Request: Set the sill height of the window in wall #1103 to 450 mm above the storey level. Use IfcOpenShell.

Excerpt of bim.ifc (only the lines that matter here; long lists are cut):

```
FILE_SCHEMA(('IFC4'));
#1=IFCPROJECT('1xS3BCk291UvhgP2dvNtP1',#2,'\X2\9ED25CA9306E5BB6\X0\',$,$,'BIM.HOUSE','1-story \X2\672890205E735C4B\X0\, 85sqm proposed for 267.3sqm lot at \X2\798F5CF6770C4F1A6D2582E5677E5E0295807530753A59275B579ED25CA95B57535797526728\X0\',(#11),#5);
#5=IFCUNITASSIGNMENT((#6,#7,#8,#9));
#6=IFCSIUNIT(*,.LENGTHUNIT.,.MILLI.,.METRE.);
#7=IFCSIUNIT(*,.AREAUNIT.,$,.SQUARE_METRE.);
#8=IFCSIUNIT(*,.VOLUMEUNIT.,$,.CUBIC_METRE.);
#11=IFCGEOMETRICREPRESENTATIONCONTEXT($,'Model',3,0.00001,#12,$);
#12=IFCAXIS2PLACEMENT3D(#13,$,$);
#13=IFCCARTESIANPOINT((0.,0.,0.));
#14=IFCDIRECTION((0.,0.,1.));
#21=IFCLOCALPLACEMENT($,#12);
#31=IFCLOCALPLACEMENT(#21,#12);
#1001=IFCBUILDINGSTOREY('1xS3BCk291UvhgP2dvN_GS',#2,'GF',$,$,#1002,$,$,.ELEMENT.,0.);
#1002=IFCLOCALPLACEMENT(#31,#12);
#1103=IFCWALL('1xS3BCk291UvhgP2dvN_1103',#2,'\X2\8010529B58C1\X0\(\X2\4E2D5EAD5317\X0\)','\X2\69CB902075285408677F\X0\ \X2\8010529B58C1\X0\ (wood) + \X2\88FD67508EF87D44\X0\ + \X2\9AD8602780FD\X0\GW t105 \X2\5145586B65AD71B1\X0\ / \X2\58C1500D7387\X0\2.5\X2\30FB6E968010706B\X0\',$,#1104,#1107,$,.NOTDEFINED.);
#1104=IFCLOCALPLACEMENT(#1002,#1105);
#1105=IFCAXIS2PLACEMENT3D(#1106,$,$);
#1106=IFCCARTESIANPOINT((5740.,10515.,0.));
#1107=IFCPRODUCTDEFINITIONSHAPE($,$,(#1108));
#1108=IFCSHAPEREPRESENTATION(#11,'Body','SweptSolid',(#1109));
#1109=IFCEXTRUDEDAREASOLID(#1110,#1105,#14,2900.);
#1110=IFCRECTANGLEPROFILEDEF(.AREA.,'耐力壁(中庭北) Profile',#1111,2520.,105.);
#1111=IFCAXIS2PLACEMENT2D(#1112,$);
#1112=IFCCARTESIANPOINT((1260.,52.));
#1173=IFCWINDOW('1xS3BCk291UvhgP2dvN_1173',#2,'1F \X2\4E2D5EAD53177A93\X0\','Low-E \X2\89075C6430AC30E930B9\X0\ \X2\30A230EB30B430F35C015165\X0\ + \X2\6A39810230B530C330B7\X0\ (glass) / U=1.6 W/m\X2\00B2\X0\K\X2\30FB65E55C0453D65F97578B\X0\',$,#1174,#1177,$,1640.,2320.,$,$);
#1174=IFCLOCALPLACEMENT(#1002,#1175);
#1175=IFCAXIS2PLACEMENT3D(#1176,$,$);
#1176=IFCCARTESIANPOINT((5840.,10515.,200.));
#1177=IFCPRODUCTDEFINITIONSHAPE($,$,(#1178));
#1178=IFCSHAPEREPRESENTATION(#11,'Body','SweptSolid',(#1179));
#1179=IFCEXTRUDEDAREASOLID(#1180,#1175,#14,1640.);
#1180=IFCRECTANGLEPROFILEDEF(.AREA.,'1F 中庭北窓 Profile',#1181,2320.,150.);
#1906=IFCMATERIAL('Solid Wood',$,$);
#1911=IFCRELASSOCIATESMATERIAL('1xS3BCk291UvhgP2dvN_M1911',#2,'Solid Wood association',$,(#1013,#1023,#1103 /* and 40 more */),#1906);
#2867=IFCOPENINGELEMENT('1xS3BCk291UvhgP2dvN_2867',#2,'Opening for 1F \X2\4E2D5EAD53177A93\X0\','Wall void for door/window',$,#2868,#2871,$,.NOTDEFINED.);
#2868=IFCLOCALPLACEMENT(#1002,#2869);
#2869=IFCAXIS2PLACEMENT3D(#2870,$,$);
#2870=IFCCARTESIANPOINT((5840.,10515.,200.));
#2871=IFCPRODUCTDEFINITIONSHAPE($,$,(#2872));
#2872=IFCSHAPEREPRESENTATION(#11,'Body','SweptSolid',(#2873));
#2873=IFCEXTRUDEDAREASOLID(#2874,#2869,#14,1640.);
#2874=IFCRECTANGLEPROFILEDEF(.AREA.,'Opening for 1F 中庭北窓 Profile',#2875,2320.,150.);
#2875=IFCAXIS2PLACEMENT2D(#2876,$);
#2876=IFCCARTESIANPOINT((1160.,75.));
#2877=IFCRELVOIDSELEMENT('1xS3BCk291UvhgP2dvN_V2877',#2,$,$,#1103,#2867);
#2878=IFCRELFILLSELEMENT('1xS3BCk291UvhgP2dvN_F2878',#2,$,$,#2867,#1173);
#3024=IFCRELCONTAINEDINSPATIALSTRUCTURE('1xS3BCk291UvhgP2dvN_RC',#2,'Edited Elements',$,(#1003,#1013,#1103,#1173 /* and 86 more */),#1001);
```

```python
import numpy as np
import ifcopenshell
import ifcopenshell.api.geometry
import ifcopenshell.geom
import ifcopenshell.util.element
import ifcopenshell.util.placement
import ifcopenshell.util.shape
import ifcopenshell.util.unit

model = ifcopenshell.open("bim.ifc")
unit_scale = ifcopenshell.util.unit.calculate_unit_scale(model)

window = model.by_guid("1xS3BCk291UvhgP2dvN_1173")
opening = window.FillsVoids[0].RelatingOpeningElement
storey = ifcopenshell.util.element.get_container(window, ifc_class="IfcBuildingStorey")
level = ifcopenshell.util.placement.get_local_placement(storey.ObjectPlacement)[2, 3]

# The opening's origin need not be at the sill, so measure its lowest point.
shape = ifcopenshell.geom.create_shape(ifcopenshell.geom.settings(), opening)
bottom = ifcopenshell.util.shape.get_shape_bottom_elevation(shape, shape.geometry) / unit_scale
dz = level + 0.45 / unit_scale - bottom

shift = np.array([0.0, 0.0, dz])
# The window is not placed relative to its opening, so move both.
for product in (opening, window):
    matrix = ifcopenshell.util.placement.get_local_placement(product.ObjectPlacement)
    matrix[:3, 3] += shift
    ifcopenshell.api.geometry.edit_object_placement(model, product=product, matrix=matrix, is_si=False)

print(f"moved by {dz * unit_scale:+.3f} m")

model.write("bim_v2.ifc")
```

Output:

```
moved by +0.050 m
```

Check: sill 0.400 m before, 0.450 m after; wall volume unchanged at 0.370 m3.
